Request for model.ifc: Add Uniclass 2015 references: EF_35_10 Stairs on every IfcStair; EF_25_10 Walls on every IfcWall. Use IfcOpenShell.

First a look at what the model holds.

```python
import ifcopenshell

model = ifcopenshell.open("model.ifc")
print(model.schema)
print("classifications:", [c.Name for c in model.by_type("IfcClassification")])
for ifc_class in ("IfcDoor", "IfcRoof", "IfcStair", "IfcWall", "IfcWindow"):
    print(ifc_class, len(model.by_type(ifc_class)))
```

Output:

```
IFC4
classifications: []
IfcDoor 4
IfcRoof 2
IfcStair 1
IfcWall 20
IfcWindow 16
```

```python
import ifcopenshell
import ifcopenshell.api.classification

model = ifcopenshell.open("model.ifc")

system = ifcopenshell.api.classification.add_classification(model, classification="Uniclass 2015")

codes = {
    "IfcStair": ("EF_35_10", "Stairs"),
    "IfcWall": ("EF_25_10", "Walls"),
}
for ifc_class, (code, name) in codes.items():
    products = model.by_type(ifc_class)
    ifcopenshell.api.classification.add_reference(
        model, products=products, classification=system, identification=code, name=name
    )
    print(code, len(products))

model.write("model-out.ifc")
```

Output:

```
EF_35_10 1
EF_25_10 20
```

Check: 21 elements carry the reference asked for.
